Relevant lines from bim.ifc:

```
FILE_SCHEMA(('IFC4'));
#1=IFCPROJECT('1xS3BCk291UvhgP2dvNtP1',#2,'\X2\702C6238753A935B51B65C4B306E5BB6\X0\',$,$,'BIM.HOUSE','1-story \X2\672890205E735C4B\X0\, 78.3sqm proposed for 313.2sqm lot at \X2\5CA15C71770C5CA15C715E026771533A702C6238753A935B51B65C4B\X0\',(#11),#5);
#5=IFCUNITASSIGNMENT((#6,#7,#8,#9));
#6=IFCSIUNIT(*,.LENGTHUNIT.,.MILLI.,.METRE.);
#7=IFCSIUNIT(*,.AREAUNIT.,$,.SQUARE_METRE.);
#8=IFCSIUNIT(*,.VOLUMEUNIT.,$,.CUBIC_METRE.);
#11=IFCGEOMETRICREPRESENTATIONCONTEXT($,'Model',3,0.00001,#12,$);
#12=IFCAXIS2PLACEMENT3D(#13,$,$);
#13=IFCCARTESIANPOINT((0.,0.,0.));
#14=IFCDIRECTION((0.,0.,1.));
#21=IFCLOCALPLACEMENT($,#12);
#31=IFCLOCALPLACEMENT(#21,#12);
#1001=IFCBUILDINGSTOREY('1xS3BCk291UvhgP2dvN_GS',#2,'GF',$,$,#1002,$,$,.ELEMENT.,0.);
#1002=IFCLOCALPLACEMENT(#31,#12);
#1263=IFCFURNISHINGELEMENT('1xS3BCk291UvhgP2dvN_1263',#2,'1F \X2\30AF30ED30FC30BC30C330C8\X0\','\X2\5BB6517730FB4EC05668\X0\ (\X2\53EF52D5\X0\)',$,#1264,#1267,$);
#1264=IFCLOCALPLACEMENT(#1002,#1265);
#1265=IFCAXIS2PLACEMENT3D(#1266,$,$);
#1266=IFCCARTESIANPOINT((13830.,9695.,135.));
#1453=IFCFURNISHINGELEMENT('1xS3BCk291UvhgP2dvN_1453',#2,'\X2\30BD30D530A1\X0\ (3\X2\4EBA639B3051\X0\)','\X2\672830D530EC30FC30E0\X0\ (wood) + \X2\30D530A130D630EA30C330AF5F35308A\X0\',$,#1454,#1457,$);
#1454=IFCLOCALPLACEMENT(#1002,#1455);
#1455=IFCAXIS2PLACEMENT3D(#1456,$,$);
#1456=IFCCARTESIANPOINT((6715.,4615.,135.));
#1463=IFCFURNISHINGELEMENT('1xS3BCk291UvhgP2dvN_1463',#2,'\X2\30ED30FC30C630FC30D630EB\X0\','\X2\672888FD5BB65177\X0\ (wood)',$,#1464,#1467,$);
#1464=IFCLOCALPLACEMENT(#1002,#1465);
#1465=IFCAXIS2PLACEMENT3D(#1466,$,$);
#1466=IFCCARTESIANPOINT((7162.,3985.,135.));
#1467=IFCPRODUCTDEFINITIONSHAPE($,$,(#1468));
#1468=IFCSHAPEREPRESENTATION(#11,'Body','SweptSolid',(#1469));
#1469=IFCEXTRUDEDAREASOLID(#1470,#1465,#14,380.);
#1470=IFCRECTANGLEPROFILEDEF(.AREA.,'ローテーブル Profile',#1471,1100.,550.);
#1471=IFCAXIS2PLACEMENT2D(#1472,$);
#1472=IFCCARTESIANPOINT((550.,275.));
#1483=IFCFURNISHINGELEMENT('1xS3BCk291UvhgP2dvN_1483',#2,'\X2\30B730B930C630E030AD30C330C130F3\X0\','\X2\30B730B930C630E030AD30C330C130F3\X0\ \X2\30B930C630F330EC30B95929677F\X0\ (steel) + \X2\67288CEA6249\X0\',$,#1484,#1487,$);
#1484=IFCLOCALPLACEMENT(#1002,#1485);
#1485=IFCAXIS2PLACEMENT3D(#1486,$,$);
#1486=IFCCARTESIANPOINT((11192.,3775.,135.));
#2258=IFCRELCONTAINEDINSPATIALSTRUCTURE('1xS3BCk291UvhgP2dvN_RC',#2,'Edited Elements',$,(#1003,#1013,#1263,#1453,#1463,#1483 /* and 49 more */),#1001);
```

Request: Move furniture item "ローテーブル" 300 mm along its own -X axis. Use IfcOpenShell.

```python
import ifcopenshell
import ifcopenshell.api.geometry
import ifcopenshell.util.placement
import ifcopenshell.util.unit

model = ifcopenshell.open("bim.ifc")
unit_scale = ifcopenshell.util.unit.calculate_unit_scale(model)

item = model.by_guid("1xS3BCk291UvhgP2dvN_1463")
matrix = ifcopenshell.util.placement.get_local_placement(item.ObjectPlacement)
matrix[:3, 3] -= matrix[:3, 0] * 0.3 / unit_scale
ifcopenshell.api.geometry.edit_object_placement(model, product=item, matrix=matrix, is_si=False)

print(ifcopenshell.util.placement.get_local_placement(item.ObjectPlacement).round(3) + 0.0)

model.write("bim-out.ifc")
```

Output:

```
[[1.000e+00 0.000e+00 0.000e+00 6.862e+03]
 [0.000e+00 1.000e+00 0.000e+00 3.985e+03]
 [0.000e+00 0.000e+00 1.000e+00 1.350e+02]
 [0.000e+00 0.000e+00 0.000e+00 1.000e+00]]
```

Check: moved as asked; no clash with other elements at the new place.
